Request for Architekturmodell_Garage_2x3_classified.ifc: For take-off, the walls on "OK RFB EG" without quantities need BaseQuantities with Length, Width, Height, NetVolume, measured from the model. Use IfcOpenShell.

First a look at what the model holds.

```python
import ifcopenshell
import ifcopenshell.util.element
import ifcopenshell.util.unit

model = ifcopenshell.open("Architekturmodell_Garage_2x3_classified.ifc")
print(model.schema)
for unit_type in ("LENGTHUNIT", "AREAUNIT", "VOLUMEUNIT"):
    print(unit_type, ifcopenshell.util.unit.calculate_unit_scale(model, unit_type))
storey = next(s for s in model.by_type("IfcBuildingStorey") if s.Name == "OK RFB EG")
walls = [e for e in ifcopenshell.util.element.get_decomposition(storey) if e.is_a("IfcWall")]
for e in sorted(walls, key=lambda e: e.id()):
    print(e.id(), e.is_a(), e.Name, list(ifcopenshell.util.element.get_psets(e, qtos_only=True)), sep=" | ")
```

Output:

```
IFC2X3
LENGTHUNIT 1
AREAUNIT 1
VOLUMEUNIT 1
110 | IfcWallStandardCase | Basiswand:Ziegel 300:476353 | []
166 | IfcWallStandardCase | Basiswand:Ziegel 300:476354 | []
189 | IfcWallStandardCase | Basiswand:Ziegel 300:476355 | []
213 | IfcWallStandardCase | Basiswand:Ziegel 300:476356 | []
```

```python
import ifcopenshell
import ifcopenshell.api.pset
import ifcopenshell.geom
import ifcopenshell.util.element
import ifcopenshell.util.shape
import ifcopenshell.util.unit

model = ifcopenshell.open("Architekturmodell_Garage_2x3_classified.ifc")
unit_scale = ifcopenshell.util.unit.calculate_unit_scale(model)
volume_scale = ifcopenshell.util.unit.calculate_unit_scale(model, "VOLUMEUNIT")
settings = ifcopenshell.geom.settings()

storey = next(s for s in model.by_type("IfcBuildingStorey") if s.Name == "OK RFB EG")
walls = [e for e in ifcopenshell.util.element.get_decomposition(storey) if e.is_a("IfcWall")]

for e in sorted(walls, key=lambda e: e.id()):
    if ifcopenshell.util.element.get_psets(e, qtos_only=True, should_inherit=False):
        continue
    # Geometry comes back in metres, in the element's own axes.
    shape = ifcopenshell.geom.create_shape(settings, e)
    values = {
        "Length": ifcopenshell.util.shape.get_x(shape.geometry) / unit_scale,
        "Width": ifcopenshell.util.shape.get_y(shape.geometry) / unit_scale,
        "Height": ifcopenshell.util.shape.get_z(shape.geometry) / unit_scale,
        "NetVolume": ifcopenshell.util.shape.get_volume(shape.geometry) / volume_scale,
    }
    qto = ifcopenshell.api.pset.add_qto(model, product=e, name="BaseQuantities")
    ifcopenshell.api.pset.edit_qto(model, qto=qto, properties=values)
    print(e.id(), {k: round(v, 3) for k, v in values.items()})

model.write("Architekturmodell_Garage_2x3_classified_rev.ifc")
```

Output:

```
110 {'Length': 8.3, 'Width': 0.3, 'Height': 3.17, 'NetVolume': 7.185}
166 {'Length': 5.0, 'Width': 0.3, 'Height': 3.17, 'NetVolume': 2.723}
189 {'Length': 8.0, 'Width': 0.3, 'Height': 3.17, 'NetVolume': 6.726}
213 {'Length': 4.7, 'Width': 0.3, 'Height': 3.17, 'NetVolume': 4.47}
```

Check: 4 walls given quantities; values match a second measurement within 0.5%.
